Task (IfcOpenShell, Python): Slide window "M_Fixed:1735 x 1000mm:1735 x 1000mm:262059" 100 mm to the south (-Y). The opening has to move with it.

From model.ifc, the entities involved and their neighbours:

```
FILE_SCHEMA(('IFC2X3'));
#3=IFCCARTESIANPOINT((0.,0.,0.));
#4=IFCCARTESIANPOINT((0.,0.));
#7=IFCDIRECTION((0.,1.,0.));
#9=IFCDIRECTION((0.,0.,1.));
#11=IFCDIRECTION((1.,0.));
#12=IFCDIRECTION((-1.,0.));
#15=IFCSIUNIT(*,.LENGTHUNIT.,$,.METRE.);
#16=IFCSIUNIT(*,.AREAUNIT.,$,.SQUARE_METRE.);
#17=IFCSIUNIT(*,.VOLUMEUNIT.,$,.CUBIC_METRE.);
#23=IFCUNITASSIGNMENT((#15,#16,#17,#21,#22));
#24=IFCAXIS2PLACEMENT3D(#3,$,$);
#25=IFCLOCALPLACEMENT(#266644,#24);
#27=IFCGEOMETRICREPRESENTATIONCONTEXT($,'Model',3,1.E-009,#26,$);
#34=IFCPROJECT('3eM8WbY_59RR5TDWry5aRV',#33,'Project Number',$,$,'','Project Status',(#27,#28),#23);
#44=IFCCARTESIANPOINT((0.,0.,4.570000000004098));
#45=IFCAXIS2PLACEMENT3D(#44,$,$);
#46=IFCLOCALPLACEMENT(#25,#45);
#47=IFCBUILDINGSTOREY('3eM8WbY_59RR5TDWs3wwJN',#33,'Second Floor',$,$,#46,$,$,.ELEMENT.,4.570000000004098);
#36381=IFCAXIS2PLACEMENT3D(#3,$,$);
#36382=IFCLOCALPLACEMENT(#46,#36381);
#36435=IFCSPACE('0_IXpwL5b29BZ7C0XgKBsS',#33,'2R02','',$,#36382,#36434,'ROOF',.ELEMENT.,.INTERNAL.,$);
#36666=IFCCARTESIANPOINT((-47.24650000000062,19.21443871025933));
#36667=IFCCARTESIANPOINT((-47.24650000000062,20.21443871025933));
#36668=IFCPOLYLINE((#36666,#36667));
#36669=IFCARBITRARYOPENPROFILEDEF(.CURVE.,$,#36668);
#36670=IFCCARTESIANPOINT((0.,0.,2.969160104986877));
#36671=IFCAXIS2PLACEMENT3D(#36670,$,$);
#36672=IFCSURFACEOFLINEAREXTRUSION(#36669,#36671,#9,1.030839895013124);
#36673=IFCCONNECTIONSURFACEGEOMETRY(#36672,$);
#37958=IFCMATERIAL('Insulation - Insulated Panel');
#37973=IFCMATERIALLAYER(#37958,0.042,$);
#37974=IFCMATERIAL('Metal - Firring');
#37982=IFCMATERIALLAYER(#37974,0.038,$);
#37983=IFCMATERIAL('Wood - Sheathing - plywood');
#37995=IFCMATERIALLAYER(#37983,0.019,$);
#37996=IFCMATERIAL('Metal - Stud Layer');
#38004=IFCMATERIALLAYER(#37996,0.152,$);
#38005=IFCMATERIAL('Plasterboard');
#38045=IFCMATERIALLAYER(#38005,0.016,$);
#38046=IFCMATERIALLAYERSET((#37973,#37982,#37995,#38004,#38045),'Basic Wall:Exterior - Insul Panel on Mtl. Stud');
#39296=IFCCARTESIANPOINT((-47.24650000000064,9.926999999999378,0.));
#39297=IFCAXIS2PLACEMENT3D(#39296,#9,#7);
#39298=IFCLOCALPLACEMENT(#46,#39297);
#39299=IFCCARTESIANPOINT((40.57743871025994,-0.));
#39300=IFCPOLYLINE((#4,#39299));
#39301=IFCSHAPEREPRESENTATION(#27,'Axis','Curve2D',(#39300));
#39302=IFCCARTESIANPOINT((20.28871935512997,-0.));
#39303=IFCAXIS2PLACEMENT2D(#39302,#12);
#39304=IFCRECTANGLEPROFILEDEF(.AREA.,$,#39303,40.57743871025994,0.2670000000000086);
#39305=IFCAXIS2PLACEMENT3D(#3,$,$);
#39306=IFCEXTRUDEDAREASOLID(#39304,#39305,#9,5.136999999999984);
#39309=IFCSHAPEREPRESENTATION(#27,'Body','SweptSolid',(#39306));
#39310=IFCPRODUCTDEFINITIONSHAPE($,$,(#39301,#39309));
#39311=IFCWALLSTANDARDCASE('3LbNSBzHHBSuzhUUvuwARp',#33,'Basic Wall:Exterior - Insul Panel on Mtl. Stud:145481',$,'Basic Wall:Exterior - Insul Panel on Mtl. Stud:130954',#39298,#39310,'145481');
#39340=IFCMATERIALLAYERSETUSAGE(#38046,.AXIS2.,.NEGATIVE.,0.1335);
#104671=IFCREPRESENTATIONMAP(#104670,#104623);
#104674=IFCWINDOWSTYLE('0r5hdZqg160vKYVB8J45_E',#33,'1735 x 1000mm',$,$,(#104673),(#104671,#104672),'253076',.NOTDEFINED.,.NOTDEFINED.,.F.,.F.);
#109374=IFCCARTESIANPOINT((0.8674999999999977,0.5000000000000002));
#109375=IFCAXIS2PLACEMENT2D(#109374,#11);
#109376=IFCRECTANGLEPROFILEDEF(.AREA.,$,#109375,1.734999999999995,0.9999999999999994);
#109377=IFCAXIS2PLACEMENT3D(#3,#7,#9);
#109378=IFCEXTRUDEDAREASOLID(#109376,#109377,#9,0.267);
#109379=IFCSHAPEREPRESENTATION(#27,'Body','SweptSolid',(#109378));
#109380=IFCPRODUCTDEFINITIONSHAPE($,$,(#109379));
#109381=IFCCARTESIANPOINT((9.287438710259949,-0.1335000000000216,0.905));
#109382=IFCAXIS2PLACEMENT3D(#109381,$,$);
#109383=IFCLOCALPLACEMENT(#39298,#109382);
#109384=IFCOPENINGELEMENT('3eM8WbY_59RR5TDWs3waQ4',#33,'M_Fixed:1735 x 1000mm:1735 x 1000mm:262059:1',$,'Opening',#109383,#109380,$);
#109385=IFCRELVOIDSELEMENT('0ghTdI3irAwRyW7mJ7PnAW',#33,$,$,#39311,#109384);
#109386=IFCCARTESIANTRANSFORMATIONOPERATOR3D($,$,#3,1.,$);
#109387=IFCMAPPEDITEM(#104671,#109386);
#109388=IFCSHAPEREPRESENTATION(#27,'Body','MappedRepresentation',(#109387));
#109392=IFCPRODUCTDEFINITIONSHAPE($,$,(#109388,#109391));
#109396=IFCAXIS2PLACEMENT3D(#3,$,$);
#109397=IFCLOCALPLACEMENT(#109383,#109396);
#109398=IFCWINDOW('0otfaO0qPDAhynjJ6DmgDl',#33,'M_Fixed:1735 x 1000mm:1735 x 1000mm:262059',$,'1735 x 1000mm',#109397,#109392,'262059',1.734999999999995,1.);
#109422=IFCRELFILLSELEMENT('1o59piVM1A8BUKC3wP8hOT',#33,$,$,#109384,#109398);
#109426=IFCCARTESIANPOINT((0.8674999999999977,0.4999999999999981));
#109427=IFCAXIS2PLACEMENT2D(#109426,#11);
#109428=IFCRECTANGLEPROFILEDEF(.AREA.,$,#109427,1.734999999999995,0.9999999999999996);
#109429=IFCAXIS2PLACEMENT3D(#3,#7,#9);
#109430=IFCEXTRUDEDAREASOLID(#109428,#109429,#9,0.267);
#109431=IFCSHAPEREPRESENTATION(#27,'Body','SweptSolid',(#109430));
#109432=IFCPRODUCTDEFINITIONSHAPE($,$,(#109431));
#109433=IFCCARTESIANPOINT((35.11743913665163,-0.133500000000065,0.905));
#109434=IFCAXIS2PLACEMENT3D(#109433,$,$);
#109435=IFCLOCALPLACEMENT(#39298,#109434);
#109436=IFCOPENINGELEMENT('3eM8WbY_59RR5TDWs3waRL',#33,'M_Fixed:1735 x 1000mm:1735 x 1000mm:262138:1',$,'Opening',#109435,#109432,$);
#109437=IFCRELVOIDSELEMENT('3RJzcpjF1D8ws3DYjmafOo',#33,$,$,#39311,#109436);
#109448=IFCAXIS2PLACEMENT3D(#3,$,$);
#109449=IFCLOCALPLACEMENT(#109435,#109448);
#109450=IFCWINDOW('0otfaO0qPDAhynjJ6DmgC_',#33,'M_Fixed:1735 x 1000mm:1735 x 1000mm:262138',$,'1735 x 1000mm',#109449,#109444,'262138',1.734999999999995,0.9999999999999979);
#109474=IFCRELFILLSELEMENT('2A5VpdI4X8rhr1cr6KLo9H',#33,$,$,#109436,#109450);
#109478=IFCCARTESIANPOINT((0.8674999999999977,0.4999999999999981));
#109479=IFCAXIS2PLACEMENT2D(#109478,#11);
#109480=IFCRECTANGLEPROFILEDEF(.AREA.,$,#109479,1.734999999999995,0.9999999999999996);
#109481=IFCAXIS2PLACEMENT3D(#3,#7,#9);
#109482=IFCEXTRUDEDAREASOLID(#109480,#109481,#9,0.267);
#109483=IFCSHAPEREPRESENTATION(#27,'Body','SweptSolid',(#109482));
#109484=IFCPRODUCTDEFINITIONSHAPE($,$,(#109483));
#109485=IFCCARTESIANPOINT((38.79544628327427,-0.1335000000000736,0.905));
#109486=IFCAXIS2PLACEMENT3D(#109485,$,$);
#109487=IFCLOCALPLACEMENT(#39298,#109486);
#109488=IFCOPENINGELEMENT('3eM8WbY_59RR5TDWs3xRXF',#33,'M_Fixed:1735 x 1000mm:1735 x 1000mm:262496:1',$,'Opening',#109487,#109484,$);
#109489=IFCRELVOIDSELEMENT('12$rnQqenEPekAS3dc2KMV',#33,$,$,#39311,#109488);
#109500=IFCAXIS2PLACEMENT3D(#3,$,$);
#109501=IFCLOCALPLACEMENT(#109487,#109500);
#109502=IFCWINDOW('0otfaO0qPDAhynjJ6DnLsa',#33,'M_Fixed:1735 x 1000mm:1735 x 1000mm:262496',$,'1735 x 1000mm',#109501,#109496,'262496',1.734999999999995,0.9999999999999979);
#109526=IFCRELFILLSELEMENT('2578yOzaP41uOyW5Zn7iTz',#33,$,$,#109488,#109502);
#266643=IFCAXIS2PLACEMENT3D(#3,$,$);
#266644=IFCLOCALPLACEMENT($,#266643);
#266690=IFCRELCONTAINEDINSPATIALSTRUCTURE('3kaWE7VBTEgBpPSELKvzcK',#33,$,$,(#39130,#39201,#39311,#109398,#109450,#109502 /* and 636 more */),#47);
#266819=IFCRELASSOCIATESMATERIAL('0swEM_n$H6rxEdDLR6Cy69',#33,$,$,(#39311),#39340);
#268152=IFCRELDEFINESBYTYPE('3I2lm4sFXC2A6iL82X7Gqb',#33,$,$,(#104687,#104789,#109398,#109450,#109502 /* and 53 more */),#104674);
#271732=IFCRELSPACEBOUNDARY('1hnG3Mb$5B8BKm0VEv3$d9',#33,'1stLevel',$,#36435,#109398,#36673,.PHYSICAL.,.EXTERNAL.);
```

```python
import numpy as np
import ifcopenshell
import ifcopenshell.api.geometry
import ifcopenshell.util.placement

model = ifcopenshell.open("model.ifc")

window = model.by_guid("0otfaO0qPDAhynjJ6DmgDl")
opening = window.FillsVoids[0].RelatingOpeningElement
wall = opening.VoidsElements[0].RelatingBuildingElement

wall_matrix = ifcopenshell.util.placement.get_local_placement(wall.ObjectPlacement)
shift = wall_matrix[:3, 0] * -0.1
before = ifcopenshell.util.placement.get_local_placement(window.ObjectPlacement)[:3, 3].copy()

# The window is placed relative to its opening, so it follows when the opening moves.
matrix = ifcopenshell.util.placement.get_local_placement(opening.ObjectPlacement)
matrix[:3, 3] += shift
ifcopenshell.api.geometry.edit_object_placement(
    model, product=opening, matrix=matrix, is_si=False, should_transform_children=True
)

# Space boundary surfaces are stored in each space's coordinates; move them too.
for rel in window.ProvidesBoundaries:
    if not rel.ConnectionGeometry:
        continue
    surface = rel.ConnectionGeometry.SurfaceOnRelatingElement
    space_matrix = ifcopenshell.util.placement.get_local_placement(rel.RelatingSpace.ObjectPlacement)
    point = np.array(surface.Position.Location.Coordinates) + space_matrix[:3, :3].T @ shift
    surface.Position = model.createIfcAxis2Placement3D(
        model.createIfcCartesianPoint(point.tolist()), surface.Position.Axis, surface.Position.RefDirection
    )

after = ifcopenshell.util.placement.get_local_placement(window.ObjectPlacement)[:3, 3]
print("window moved by", (after - before).round(3) + 0.0)

model.write("model-out.ifc")
```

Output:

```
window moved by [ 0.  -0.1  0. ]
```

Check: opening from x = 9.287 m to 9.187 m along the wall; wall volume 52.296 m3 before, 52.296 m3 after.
